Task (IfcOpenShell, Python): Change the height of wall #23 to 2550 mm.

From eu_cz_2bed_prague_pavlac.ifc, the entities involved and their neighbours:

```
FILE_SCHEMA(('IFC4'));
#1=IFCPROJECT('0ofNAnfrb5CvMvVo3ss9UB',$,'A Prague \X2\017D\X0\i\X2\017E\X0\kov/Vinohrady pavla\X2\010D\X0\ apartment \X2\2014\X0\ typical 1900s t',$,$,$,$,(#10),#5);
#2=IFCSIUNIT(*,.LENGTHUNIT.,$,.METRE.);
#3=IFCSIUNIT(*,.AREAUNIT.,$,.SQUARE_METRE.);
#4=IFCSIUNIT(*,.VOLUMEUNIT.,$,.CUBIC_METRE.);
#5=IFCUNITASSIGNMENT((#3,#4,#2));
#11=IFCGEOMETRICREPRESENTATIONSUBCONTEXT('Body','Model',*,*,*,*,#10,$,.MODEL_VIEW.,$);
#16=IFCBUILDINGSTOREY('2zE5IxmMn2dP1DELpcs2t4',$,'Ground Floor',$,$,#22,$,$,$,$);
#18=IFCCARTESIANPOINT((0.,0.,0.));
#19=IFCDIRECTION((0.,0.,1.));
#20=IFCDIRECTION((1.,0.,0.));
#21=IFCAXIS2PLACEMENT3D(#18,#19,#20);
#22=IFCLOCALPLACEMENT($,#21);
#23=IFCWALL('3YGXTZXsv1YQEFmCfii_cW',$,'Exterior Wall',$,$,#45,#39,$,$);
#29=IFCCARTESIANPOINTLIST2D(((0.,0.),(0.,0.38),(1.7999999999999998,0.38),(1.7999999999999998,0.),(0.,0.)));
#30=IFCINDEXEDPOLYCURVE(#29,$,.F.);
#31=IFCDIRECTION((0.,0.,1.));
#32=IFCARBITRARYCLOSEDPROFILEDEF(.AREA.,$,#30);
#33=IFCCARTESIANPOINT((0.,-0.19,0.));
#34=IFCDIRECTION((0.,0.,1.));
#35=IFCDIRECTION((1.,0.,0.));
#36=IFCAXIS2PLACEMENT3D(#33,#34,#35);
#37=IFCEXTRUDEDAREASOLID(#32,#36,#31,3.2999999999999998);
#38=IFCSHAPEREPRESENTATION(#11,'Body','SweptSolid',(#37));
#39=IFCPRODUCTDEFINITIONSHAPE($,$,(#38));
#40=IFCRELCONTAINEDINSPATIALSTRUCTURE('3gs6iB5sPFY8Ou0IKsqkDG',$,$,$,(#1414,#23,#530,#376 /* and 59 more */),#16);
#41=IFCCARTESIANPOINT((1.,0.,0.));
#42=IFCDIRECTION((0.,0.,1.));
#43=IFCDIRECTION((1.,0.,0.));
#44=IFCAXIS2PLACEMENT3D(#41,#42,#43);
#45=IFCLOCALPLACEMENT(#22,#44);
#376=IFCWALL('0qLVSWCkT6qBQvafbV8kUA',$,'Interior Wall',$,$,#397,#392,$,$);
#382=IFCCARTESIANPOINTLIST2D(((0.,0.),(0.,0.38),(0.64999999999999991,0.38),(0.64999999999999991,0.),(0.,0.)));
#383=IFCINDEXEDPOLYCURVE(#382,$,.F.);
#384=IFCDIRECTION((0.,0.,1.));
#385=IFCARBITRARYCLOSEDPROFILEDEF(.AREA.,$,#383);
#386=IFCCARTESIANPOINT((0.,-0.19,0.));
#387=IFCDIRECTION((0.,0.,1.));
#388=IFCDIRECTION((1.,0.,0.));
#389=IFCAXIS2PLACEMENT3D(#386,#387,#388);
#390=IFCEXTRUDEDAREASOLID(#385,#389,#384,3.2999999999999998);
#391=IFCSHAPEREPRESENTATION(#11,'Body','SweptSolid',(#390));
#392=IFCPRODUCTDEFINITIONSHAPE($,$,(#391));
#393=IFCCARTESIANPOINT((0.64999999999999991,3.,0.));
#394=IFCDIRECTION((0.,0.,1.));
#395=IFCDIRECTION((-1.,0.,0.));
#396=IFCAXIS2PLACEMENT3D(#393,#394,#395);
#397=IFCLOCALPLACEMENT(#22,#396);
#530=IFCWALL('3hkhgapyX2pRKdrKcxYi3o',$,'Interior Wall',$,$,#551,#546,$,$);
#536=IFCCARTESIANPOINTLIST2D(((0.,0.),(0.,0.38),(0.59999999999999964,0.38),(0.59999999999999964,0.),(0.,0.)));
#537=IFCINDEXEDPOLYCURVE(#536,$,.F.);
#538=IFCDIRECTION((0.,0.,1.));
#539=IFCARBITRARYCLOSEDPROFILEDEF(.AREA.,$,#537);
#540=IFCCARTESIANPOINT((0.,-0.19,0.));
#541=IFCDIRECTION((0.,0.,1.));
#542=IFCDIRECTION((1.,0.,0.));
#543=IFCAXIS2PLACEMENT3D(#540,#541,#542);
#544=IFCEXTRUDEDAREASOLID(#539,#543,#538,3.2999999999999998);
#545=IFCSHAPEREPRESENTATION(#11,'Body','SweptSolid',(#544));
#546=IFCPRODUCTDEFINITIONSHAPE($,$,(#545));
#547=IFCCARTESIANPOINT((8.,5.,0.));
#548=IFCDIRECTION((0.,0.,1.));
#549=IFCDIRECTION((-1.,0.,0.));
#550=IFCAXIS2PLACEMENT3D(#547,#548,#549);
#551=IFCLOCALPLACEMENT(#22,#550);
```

```python
import ifcopenshell
import ifcopenshell.geom
import ifcopenshell.util.representation
import ifcopenshell.util.shape
import ifcopenshell.util.unit

model = ifcopenshell.open("eu_cz_2bed_prague_pavlac.ifc")
unit_scale = ifcopenshell.util.unit.calculate_unit_scale(model)
settings = ifcopenshell.geom.settings()


def volume(element):
    """Net volume in cubic metres, openings subtracted."""
    shape = ifcopenshell.geom.create_shape(settings, element)
    return ifcopenshell.util.shape.get_volume(shape.geometry)


wall = model.by_guid("3YGXTZXsv1YQEFmCfii_cW")
before = volume(wall)

body = ifcopenshell.util.representation.get_representation(wall, "Model", "Body")
solid = body.Items[0]
old_height = solid.Depth
solid.Depth = 2.55 / unit_scale
after = volume(wall)

print(f"height {old_height:g} -> {solid.Depth:g}, volume {before:.3f} -> {after:.3f} m3")

model.write("eu_cz_2bed_prague_pavlac-out.ifc")
```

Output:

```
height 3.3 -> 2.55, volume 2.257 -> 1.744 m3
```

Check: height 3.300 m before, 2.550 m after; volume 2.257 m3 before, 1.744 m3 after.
